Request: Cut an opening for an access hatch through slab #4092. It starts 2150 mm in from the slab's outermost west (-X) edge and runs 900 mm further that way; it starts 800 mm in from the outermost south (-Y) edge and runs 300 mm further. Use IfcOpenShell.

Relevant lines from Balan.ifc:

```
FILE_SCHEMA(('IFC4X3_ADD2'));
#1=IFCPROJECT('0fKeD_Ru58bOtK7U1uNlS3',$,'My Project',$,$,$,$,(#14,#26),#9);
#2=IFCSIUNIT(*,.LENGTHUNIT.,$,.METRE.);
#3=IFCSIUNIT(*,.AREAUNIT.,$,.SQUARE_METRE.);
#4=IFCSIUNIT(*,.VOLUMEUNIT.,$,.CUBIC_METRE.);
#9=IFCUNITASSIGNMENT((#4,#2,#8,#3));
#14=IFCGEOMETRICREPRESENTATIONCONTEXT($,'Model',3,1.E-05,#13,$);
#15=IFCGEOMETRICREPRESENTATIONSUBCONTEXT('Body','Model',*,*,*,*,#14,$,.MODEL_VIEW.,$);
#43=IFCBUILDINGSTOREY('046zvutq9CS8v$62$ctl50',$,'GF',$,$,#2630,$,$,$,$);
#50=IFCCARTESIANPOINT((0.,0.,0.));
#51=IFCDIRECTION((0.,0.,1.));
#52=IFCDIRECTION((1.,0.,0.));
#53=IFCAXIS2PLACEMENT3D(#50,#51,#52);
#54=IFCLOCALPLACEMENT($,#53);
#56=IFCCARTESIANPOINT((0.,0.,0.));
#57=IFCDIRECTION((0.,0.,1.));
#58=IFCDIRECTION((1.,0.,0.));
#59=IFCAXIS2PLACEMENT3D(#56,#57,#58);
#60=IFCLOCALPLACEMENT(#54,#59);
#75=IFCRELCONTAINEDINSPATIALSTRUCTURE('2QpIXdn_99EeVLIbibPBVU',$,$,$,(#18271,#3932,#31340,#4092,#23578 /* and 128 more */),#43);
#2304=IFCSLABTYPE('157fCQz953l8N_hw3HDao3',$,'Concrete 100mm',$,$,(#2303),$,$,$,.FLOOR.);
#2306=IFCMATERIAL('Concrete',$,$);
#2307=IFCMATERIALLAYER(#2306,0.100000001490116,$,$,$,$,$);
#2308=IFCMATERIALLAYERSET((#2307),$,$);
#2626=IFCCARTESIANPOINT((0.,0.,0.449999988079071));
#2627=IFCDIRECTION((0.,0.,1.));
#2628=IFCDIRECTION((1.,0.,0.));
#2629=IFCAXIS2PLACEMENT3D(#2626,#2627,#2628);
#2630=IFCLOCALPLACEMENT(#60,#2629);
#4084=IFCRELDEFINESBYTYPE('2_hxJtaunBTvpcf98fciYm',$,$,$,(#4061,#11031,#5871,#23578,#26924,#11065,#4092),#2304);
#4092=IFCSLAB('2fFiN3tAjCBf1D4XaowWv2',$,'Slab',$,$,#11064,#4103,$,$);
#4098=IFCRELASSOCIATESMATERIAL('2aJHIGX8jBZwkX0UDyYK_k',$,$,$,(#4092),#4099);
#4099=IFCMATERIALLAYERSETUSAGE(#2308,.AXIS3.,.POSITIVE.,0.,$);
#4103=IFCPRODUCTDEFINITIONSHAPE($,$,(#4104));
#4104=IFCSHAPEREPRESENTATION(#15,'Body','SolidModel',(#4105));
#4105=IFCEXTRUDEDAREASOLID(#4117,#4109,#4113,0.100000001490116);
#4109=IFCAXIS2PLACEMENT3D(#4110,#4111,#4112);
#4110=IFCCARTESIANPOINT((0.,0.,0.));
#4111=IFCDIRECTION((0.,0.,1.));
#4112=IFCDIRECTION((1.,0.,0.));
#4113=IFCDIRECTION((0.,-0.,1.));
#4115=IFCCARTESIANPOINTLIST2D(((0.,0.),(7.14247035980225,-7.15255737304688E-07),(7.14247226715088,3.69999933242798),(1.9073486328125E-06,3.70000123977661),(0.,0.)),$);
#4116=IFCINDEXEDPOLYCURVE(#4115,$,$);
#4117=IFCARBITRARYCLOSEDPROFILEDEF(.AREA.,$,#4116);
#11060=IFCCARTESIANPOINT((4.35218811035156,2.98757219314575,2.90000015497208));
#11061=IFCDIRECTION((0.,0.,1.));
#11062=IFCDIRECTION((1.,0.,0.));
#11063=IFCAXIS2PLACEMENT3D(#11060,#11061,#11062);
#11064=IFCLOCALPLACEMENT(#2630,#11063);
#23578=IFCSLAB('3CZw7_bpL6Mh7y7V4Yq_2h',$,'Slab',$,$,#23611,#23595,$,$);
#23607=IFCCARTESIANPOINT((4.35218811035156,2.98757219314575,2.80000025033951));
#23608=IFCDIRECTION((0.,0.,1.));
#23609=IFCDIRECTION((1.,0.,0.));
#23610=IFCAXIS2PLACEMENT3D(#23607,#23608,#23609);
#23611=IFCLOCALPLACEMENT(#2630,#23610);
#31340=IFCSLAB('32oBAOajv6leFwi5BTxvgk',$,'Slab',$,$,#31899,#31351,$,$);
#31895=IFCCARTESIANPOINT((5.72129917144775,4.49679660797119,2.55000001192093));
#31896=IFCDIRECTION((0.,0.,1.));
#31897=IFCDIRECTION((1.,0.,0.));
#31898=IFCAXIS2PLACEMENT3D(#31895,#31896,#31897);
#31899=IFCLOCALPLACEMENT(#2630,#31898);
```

```python
import numpy as np
import ifcopenshell
import ifcopenshell.api.feature
import ifcopenshell.api.geometry
import ifcopenshell.api.root
import ifcopenshell.geom
import ifcopenshell.util.placement
import ifcopenshell.util.representation
import ifcopenshell.util.shape
import ifcopenshell.util.unit

model = ifcopenshell.open("Balan.ifc")
unit_scale = ifcopenshell.util.unit.calculate_unit_scale(model)
settings = ifcopenshell.geom.settings()


def volume(element):
    """Net volume in cubic metres, openings subtracted."""
    shape = ifcopenshell.geom.create_shape(settings, element)
    return ifcopenshell.util.shape.get_volume(shape.geometry)


slab = model.by_guid("2fFiN3tAjCBf1D4XaowWv2")
before = volume(slab)

# Extent in the slab's own axes, in metres. The edges named are its -X and -Y sides.
slab_shape = ifcopenshell.geom.create_shape(settings, slab)
vertices = ifcopenshell.util.shape.get_vertices(slab_shape.geometry)
x_min, y_min, bottom = vertices.min(axis=0)
top = vertices[:, 2].max()

opening = ifcopenshell.api.root.create_entity(model, ifc_class="IfcOpeningElement", name="Access hatch opening", predefined_type="OPENING")
context = ifcopenshell.util.representation.get_context(model, "Model", "Body", "MODEL_VIEW")
width, depth = 0.9, 0.3
outline = [(0.0, 0.0), (width, 0.0), (width, depth), (0.0, depth), (0.0, 0.0)]
# Overshoot both faces by 50 mm so the cut is clean.
shape = ifcopenshell.api.geometry.add_slab_representation(
    model, context=context, depth=top - bottom + 0.1, polyline=outline
)
ifcopenshell.api.geometry.assign_representation(model, product=opening, representation=shape)

matrix = ifcopenshell.util.placement.get_local_placement(slab.ObjectPlacement)
matrix[:, 3] = matrix @ np.append(np.array([x_min + 2.15, y_min + 0.8, bottom - 0.05]) / unit_scale, 1.0)
ifcopenshell.api.geometry.edit_object_placement(model, product=opening, matrix=matrix, is_si=False)
ifcopenshell.api.feature.add_feature(model, feature=opening, element=slab)

after = volume(slab)

print(f"slab volume {before:.3f} -> {after:.3f} m3")

model.write("Balan_edited.ifc")
```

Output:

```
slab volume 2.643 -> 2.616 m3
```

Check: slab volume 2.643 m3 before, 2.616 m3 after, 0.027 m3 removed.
